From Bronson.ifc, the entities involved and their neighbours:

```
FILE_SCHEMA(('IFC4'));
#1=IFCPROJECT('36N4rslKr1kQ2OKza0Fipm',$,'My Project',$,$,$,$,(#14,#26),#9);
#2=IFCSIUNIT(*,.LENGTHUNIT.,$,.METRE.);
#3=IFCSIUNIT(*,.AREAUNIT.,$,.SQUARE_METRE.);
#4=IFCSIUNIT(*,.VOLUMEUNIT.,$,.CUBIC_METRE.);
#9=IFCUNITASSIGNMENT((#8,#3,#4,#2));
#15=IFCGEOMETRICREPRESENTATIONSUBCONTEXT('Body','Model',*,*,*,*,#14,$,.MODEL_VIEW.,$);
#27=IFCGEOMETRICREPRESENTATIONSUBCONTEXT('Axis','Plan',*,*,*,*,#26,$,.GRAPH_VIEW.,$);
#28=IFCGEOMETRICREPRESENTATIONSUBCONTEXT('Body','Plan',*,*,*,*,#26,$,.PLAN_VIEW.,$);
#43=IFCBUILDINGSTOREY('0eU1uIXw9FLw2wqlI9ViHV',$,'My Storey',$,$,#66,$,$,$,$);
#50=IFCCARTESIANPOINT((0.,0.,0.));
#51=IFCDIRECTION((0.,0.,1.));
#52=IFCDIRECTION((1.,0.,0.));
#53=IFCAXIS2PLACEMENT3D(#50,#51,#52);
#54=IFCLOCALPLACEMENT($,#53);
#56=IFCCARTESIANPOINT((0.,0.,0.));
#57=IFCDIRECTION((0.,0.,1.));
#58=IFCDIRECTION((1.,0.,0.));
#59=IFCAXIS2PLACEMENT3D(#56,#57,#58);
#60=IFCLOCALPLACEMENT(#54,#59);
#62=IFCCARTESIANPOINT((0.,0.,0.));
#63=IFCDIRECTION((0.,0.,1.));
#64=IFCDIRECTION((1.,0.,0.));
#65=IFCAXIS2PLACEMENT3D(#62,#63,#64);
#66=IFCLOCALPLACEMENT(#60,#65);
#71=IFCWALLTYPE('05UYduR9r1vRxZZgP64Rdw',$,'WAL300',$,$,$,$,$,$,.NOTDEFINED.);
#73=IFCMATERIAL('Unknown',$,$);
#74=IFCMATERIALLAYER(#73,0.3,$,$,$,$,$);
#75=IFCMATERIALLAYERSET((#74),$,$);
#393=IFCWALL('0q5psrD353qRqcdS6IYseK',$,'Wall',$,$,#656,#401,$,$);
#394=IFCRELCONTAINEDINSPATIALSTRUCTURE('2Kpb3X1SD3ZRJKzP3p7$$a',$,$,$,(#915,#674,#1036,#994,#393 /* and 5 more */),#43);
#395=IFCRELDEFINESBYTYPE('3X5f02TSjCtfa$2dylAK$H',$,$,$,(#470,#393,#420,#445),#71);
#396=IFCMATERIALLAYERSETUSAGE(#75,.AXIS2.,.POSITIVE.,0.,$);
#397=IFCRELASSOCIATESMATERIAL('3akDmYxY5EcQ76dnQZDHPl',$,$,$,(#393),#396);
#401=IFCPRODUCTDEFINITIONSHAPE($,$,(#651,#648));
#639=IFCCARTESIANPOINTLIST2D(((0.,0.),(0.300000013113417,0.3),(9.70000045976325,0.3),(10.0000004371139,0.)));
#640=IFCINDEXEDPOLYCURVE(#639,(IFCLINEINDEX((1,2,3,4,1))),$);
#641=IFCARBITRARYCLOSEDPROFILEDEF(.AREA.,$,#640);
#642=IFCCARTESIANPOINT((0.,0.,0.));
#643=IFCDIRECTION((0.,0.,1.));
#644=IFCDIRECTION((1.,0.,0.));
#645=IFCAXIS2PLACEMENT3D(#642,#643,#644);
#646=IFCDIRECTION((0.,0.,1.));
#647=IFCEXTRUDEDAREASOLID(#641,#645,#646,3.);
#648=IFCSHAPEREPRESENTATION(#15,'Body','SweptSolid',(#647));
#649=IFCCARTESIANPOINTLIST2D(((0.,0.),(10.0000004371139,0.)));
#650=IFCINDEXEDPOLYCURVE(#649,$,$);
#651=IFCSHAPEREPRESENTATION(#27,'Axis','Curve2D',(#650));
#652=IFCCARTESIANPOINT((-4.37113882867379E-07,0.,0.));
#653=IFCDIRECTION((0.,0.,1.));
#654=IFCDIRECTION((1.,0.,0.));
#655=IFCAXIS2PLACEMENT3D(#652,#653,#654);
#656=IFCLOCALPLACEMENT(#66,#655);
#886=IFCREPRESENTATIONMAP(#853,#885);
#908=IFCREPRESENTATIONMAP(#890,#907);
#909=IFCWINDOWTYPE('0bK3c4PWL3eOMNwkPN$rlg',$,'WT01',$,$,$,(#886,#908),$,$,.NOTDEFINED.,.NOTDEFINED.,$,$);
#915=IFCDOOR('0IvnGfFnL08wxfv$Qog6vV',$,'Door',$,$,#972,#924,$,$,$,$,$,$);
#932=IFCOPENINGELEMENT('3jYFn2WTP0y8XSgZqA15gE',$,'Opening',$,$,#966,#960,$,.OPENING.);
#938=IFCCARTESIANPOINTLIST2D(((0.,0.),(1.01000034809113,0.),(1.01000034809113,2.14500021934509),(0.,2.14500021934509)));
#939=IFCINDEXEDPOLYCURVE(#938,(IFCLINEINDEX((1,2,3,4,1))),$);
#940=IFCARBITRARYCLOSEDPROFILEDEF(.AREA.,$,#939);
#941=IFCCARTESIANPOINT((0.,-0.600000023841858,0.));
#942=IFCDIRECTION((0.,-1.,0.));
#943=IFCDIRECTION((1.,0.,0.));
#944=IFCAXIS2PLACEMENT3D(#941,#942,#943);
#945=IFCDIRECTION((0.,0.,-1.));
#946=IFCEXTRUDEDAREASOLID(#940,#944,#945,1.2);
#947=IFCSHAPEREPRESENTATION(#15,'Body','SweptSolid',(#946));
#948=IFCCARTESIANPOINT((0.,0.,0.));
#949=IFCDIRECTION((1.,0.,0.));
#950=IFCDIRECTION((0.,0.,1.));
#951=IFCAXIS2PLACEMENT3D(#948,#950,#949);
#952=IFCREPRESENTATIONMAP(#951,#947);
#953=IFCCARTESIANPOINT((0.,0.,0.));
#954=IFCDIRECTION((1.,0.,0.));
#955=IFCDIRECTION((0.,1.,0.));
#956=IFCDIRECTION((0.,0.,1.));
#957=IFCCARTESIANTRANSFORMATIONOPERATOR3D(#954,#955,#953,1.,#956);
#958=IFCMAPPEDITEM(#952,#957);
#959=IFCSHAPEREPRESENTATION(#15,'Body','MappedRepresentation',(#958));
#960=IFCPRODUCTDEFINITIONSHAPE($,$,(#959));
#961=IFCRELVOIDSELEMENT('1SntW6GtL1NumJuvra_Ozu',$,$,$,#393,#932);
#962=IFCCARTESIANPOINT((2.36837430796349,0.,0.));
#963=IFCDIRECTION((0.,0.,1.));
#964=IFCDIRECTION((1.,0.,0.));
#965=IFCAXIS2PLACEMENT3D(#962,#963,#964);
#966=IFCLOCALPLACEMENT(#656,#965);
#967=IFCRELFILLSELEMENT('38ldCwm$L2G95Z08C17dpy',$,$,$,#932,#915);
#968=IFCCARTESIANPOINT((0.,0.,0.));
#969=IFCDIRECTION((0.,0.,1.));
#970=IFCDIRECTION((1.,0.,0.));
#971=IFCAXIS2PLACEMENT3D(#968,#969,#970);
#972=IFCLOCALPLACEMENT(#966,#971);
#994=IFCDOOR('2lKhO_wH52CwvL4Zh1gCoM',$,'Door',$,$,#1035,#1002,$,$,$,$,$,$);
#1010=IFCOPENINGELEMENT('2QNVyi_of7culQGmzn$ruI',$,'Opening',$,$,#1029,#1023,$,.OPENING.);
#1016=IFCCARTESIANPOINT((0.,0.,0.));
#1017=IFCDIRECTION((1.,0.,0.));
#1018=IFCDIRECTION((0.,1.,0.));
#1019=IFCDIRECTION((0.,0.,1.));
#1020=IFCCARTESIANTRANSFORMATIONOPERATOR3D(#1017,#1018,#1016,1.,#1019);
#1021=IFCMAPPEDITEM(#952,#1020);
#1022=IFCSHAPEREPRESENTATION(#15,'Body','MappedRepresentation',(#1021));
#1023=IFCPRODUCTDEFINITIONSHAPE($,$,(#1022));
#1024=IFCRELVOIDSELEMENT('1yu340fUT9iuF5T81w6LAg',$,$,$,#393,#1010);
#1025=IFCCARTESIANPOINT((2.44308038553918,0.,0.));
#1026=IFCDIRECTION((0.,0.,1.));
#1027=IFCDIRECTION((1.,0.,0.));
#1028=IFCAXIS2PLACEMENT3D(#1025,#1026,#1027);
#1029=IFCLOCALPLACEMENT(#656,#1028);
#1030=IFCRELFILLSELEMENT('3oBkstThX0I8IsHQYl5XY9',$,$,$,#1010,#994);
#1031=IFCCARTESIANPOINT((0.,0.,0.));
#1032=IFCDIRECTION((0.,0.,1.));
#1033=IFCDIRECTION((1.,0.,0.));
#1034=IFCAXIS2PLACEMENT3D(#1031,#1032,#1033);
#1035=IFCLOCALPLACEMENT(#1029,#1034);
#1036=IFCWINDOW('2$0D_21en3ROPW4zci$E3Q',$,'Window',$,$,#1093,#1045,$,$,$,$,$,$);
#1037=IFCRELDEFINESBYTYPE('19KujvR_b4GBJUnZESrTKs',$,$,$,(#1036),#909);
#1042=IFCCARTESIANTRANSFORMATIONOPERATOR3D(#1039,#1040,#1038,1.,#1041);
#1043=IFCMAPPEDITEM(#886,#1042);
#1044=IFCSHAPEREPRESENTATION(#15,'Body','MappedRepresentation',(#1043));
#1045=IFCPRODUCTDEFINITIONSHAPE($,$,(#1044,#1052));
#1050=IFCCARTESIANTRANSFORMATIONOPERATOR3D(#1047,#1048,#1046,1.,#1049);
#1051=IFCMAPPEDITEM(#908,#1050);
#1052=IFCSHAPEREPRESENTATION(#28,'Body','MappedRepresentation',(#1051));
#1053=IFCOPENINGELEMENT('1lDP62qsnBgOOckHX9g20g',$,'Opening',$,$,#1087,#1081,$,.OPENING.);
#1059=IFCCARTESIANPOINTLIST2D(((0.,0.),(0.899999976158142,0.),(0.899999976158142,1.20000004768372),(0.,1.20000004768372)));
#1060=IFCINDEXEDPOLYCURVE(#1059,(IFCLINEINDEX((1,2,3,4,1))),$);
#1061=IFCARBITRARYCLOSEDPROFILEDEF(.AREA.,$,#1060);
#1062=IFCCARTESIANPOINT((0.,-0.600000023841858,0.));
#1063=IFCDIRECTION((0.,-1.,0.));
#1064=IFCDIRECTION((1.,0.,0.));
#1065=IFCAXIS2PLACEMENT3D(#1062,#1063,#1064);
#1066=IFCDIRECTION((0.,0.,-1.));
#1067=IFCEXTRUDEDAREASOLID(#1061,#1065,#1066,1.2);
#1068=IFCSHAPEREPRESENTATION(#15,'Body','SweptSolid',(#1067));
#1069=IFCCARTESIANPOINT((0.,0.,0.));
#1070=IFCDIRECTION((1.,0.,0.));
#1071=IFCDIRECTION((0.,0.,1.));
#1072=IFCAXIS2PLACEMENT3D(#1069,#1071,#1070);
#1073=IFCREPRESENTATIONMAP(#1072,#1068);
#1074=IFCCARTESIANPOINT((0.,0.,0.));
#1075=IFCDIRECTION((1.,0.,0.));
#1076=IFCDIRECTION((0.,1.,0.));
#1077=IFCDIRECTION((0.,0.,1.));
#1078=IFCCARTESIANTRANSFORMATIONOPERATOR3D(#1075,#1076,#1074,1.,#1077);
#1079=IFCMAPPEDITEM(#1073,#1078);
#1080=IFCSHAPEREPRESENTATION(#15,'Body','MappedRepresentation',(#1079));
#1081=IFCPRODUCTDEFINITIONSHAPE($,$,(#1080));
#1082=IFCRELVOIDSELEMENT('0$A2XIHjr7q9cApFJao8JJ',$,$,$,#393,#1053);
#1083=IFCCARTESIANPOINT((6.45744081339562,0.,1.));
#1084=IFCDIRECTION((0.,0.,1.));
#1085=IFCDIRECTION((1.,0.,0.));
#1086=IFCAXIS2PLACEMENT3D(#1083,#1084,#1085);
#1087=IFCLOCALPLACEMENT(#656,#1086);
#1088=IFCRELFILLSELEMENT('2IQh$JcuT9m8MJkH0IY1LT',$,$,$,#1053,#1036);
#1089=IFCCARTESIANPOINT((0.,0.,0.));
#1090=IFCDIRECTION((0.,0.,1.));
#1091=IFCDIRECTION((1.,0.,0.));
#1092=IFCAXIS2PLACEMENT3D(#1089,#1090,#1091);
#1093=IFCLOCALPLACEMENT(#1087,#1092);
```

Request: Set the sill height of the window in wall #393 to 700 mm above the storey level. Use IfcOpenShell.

```python
import numpy as np
import ifcopenshell
import ifcopenshell.api.geometry
import ifcopenshell.geom
import ifcopenshell.util.element
import ifcopenshell.util.placement
import ifcopenshell.util.shape
import ifcopenshell.util.unit

model = ifcopenshell.open("Bronson.ifc")
unit_scale = ifcopenshell.util.unit.calculate_unit_scale(model)

window = model.by_id(1036)
opening = window.FillsVoids[0].RelatingOpeningElement
storey = ifcopenshell.util.element.get_container(window, ifc_class="IfcBuildingStorey")
level = ifcopenshell.util.placement.get_local_placement(storey.ObjectPlacement)[2, 3]

# The opening's origin need not be at the sill, so measure its lowest point.
shape = ifcopenshell.geom.create_shape(ifcopenshell.geom.settings(), opening)
bottom = ifcopenshell.util.shape.get_shape_bottom_elevation(shape, shape.geometry) / unit_scale
dz = level + 0.7 - bottom

shift = np.array([0.0, 0.0, dz])
# The window is placed relative to its opening, so it follows when the opening moves.
matrix = ifcopenshell.util.placement.get_local_placement(opening.ObjectPlacement)
matrix[:3, 3] += shift
ifcopenshell.api.geometry.edit_object_placement(
    model, product=opening, matrix=matrix, is_si=False, should_transform_children=True
)

print(f"moved by {dz * unit_scale:+.3f} m")

model.write("Bronson-out.ifc")
```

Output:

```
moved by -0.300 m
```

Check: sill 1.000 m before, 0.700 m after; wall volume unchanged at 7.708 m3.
